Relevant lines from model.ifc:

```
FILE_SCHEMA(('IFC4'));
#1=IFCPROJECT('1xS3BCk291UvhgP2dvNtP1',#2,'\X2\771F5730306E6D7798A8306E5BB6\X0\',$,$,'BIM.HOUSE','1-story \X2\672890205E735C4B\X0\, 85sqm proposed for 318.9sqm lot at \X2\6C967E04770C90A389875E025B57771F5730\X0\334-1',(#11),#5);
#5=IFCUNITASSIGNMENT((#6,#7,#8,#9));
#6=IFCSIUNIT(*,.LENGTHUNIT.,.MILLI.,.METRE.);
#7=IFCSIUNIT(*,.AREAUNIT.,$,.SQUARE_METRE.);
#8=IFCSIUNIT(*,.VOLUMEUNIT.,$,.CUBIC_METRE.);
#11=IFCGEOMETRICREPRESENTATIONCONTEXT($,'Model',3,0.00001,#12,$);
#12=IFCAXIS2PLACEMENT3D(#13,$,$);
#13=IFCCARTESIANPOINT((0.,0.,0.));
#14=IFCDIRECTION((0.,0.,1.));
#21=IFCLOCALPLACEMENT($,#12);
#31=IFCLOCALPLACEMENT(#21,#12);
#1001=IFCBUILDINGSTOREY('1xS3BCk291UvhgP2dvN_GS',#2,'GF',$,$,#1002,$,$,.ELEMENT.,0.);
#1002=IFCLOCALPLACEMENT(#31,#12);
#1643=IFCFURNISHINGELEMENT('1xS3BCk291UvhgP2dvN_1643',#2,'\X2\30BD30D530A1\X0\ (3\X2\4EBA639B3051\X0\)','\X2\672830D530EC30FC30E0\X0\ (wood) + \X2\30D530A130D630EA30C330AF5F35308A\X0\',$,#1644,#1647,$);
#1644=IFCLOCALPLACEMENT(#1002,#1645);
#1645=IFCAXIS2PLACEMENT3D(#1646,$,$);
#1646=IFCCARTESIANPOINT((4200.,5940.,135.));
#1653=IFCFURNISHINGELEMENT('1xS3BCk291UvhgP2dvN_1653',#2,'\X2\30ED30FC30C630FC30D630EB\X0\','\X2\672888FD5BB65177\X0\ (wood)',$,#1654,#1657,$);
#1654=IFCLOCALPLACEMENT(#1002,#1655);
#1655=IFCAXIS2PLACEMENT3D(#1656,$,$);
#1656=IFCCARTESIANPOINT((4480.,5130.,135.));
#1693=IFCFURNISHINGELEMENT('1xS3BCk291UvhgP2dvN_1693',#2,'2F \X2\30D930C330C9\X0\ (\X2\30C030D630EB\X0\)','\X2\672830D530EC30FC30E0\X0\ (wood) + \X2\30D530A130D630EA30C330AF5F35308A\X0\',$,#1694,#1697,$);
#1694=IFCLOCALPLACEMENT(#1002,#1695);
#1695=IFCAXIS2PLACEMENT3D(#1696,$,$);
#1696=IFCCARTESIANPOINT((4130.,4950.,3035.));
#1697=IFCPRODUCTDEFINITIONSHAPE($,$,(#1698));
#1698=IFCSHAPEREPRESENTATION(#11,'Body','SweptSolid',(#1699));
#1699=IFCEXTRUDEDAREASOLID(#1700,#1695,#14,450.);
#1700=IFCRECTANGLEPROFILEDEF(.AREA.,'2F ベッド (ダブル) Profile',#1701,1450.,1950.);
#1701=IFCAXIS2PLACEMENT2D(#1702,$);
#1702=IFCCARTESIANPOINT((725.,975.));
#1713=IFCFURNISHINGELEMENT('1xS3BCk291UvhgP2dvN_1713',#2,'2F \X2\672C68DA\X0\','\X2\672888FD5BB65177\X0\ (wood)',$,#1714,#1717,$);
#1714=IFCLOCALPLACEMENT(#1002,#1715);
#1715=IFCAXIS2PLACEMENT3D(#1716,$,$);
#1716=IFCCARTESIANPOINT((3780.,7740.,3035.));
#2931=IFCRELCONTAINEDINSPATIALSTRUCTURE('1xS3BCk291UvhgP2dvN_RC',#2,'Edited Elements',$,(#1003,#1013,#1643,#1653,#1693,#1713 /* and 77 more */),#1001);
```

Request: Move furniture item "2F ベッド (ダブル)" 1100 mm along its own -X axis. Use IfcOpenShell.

```python
import ifcopenshell
import ifcopenshell.api.geometry
import ifcopenshell.util.placement
import ifcopenshell.util.unit

model = ifcopenshell.open("model.ifc")
unit_scale = ifcopenshell.util.unit.calculate_unit_scale(model)

item = model.by_guid("1xS3BCk291UvhgP2dvN_1693")
matrix = ifcopenshell.util.placement.get_local_placement(item.ObjectPlacement)
matrix[:3, 3] -= matrix[:3, 0] * 1.1 / unit_scale
ifcopenshell.api.geometry.edit_object_placement(model, product=item, matrix=matrix, is_si=False)

print(ifcopenshell.util.placement.get_local_placement(item.ObjectPlacement).round(3) + 0.0)

model.write("model-out.ifc")
```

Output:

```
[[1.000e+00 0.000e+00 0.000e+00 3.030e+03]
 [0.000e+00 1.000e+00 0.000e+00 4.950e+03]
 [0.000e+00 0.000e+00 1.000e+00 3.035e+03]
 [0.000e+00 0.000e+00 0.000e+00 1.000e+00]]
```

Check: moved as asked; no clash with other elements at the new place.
